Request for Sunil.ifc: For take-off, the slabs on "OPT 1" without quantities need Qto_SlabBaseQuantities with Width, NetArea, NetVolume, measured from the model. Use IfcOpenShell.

First a look at what the model holds.

```python
import ifcopenshell
import ifcopenshell.util.element
import ifcopenshell.util.unit

model = ifcopenshell.open("Sunil.ifc")
print(model.schema)
for unit_type in ("LENGTHUNIT", "AREAUNIT", "VOLUMEUNIT"):
    print(unit_type, ifcopenshell.util.unit.calculate_unit_scale(model, unit_type))
storey = next(s for s in model.by_type("IfcBuildingStorey") if s.Name == "OPT 1")
slabs = [e for e in ifcopenshell.util.element.get_decomposition(storey) if e.is_a("IfcSlab")]
for e in sorted(slabs, key=lambda e: e.id()):
    print(e.id(), e.is_a(), e.Name, list(ifcopenshell.util.element.get_psets(e, qtos_only=True)), sep=" | ")
```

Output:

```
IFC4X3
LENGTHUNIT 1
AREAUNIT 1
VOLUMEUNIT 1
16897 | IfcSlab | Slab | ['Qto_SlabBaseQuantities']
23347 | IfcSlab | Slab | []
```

```python
import ifcopenshell
import ifcopenshell.api.pset
import ifcopenshell.geom
import ifcopenshell.util.element
import ifcopenshell.util.shape
import ifcopenshell.util.unit

model = ifcopenshell.open("Sunil.ifc")
unit_scale = ifcopenshell.util.unit.calculate_unit_scale(model)
area_scale = ifcopenshell.util.unit.calculate_unit_scale(model, "AREAUNIT")
volume_scale = ifcopenshell.util.unit.calculate_unit_scale(model, "VOLUMEUNIT")
settings = ifcopenshell.geom.settings()

storey = next(s for s in model.by_type("IfcBuildingStorey") if s.Name == "OPT 1")
slabs = [e for e in ifcopenshell.util.element.get_decomposition(storey) if e.is_a("IfcSlab")]

for e in sorted(slabs, key=lambda e: e.id()):
    if ifcopenshell.util.element.get_psets(e, qtos_only=True, should_inherit=False):
        continue
    # Geometry comes back in metres, in the element's own axes.
    shape = ifcopenshell.geom.create_shape(settings, e)
    values = {
        "Width": ifcopenshell.util.shape.get_z(shape.geometry) / unit_scale,
        "NetArea": ifcopenshell.util.shape.get_footprint_area(shape.geometry) / area_scale,
        "NetVolume": ifcopenshell.util.shape.get_volume(shape.geometry) / volume_scale,
    }
    qto = ifcopenshell.api.pset.add_qto(model, product=e, name="Qto_SlabBaseQuantities")
    ifcopenshell.api.pset.edit_qto(model, qto=qto, properties=values)
    print(e.id(), {k: round(v, 3) for k, v in values.items()})

model.write("Sunil_rev.ifc")
```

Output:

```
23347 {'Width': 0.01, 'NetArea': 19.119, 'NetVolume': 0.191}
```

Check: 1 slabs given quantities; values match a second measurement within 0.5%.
